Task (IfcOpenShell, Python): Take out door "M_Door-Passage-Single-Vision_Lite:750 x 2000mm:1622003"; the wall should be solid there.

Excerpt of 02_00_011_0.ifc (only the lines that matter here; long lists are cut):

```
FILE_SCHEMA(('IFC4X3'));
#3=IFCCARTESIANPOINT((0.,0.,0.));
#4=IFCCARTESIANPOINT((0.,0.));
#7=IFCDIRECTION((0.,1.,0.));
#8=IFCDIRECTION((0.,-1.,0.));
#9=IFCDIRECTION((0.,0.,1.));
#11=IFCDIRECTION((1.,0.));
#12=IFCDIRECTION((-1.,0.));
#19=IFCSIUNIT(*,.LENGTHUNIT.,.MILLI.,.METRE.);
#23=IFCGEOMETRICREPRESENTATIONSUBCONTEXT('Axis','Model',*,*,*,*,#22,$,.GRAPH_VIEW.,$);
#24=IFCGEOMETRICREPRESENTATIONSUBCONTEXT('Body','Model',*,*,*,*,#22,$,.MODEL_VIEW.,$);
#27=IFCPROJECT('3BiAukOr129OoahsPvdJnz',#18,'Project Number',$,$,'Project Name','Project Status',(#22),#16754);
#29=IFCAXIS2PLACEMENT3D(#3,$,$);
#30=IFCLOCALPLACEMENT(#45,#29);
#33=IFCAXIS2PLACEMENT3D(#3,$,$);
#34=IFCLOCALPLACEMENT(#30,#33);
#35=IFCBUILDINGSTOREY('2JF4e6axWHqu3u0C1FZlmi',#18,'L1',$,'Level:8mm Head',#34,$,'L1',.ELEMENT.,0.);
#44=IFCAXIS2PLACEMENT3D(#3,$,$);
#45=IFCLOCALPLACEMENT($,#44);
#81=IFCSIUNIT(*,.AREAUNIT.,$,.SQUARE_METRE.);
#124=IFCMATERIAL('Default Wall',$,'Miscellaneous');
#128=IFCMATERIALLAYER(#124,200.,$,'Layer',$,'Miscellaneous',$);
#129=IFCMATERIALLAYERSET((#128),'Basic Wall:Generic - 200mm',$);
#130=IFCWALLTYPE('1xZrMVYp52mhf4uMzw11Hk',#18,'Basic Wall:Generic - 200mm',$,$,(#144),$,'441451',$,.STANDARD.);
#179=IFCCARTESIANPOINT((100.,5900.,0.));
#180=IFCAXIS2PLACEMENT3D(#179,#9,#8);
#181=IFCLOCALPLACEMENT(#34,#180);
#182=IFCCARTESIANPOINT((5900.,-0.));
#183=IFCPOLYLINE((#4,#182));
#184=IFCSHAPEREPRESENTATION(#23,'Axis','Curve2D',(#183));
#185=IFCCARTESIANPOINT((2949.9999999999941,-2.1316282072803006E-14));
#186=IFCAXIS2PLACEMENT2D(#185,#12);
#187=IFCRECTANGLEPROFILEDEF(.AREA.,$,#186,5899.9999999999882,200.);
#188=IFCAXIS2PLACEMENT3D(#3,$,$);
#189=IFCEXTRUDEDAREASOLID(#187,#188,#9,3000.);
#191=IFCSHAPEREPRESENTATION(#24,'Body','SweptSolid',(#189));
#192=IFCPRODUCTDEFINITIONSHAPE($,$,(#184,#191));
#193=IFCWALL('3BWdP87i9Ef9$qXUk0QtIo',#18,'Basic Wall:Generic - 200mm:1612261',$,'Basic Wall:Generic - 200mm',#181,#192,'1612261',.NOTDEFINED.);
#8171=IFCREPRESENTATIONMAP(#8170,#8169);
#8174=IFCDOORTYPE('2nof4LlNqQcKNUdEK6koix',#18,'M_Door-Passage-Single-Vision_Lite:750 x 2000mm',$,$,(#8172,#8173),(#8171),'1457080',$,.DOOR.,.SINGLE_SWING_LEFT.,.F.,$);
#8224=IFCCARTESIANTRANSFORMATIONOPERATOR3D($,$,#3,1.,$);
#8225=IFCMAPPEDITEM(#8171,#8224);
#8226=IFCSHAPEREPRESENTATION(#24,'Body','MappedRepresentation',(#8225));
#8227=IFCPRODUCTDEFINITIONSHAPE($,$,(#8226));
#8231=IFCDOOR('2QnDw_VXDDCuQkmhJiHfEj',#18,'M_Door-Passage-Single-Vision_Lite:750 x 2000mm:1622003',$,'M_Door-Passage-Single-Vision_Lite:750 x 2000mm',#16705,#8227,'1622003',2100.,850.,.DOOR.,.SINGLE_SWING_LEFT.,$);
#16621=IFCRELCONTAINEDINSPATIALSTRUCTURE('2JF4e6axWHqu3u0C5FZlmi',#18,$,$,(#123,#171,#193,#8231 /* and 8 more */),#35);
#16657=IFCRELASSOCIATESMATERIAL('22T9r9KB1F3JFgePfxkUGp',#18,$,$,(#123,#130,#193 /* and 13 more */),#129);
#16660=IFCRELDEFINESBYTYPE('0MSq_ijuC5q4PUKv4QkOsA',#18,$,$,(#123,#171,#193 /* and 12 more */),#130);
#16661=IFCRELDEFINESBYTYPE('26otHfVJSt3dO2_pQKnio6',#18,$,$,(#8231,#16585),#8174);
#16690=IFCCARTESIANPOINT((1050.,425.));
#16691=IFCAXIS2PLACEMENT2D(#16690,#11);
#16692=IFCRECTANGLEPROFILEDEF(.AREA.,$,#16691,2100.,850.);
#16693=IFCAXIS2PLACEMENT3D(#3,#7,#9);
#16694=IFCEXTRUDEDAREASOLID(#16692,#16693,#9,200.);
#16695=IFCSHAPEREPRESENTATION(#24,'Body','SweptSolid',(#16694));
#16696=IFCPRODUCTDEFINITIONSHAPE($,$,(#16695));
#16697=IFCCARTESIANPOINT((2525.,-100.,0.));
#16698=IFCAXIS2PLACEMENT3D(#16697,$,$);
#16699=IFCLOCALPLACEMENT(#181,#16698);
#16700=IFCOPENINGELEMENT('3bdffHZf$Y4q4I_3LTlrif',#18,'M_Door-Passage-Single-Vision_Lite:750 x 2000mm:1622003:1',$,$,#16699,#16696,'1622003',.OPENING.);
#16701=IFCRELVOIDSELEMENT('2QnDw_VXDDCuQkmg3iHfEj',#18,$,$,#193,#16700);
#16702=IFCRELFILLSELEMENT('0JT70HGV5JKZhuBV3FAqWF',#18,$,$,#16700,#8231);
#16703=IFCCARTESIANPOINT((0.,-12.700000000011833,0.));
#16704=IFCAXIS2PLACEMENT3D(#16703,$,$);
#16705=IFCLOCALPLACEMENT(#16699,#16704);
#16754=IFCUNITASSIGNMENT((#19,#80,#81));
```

```python
import ifcopenshell
import ifcopenshell.api.feature
import ifcopenshell.api.root
import ifcopenshell.geom
import ifcopenshell.util.shape

model = ifcopenshell.open("02_00_011_0.ifc")
settings = ifcopenshell.geom.settings()


def volume(element):
    """Net volume in cubic metres, openings subtracted."""
    shape = ifcopenshell.geom.create_shape(settings, element)
    return ifcopenshell.util.shape.get_volume(shape.geometry)


door = model.by_id(8231)
opening = door.FillsVoids[0].RelatingOpeningElement
wall = opening.VoidsElements[0].RelatingBuildingElement
before = volume(wall)

ifcopenshell.api.root.remove_product(model, product=door)
ifcopenshell.api.feature.remove_feature(model, feature=opening)

after = volume(wall)

print(f"wall volume {before:.3f} -> {after:.3f} m3")

model.write("02_00_011_0-out.ifc")
```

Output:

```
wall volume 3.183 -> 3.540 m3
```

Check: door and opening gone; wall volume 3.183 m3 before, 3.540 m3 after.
